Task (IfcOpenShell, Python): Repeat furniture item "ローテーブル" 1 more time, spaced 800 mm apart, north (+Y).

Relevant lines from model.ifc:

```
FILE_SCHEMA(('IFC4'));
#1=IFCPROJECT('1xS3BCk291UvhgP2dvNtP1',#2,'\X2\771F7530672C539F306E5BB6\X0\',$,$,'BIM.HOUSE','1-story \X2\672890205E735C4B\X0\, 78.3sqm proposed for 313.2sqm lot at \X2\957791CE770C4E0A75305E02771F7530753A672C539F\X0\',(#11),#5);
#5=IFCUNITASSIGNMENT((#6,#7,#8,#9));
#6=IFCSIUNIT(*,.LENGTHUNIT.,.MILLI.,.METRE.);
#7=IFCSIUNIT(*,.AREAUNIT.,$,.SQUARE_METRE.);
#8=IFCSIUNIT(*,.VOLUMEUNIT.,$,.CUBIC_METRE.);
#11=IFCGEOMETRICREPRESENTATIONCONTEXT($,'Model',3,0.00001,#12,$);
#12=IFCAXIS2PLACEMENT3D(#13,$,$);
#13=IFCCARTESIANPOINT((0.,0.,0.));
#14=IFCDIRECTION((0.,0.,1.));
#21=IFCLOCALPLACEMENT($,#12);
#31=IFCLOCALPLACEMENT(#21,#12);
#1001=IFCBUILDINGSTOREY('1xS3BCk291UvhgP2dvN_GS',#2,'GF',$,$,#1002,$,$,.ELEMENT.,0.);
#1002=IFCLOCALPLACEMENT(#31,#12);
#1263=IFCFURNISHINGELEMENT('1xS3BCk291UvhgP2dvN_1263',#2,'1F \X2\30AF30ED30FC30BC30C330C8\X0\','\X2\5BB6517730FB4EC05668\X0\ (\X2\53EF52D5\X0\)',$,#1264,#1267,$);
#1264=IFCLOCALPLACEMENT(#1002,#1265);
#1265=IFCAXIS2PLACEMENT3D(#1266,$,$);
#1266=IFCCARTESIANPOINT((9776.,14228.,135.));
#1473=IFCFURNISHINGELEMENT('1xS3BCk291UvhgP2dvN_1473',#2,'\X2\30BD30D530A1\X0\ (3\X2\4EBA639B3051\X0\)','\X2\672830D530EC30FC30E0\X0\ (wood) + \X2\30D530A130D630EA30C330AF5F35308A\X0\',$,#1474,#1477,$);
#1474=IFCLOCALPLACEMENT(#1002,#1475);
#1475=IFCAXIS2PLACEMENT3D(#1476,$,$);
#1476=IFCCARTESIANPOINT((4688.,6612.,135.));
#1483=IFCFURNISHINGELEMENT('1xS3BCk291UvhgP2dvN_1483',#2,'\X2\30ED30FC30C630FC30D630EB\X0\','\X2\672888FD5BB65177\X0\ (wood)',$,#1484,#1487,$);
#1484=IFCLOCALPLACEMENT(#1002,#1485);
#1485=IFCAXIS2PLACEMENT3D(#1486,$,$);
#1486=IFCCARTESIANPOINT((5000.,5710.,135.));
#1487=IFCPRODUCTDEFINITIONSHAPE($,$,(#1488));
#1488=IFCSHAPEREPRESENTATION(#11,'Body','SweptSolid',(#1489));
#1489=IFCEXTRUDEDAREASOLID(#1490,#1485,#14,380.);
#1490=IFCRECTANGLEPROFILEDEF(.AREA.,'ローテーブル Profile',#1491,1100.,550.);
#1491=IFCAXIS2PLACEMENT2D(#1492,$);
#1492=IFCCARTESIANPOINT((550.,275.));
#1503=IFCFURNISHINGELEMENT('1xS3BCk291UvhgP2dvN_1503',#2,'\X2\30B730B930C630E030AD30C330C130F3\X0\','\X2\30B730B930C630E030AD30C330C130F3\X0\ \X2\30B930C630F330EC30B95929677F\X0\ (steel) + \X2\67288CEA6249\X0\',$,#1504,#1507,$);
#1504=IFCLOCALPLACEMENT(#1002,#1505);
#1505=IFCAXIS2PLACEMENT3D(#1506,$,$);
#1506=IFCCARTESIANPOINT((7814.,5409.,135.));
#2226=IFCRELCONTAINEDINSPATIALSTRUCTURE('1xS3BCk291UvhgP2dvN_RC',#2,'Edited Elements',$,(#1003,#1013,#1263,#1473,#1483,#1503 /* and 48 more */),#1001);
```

```python
import numpy as np
import ifcopenshell
import ifcopenshell.api.geometry
import ifcopenshell.api.root
import ifcopenshell.util.element
import ifcopenshell.util.placement

model = ifcopenshell.open("model.ifc")


def reuse_history(source, copy):
    """copy_class also copies each property set's owner history, people and application; keep the originals."""
    for rel in copy.IsDefinedBy:
        if rel.is_a("IfcRelDefinesByProperties") and (history := rel.RelatingPropertyDefinition.OwnerHistory):
            rel.RelatingPropertyDefinition.OwnerHistory = source.OwnerHistory
            ifcopenshell.util.element.remove_deep2(model, history)


source = model.by_id(1483)
base = ifcopenshell.util.placement.get_local_placement(source.ObjectPlacement)
step = np.array([0.0, 1.0, 0.0]) * 800.0

for i in range(1, 2):
    copy = ifcopenshell.api.root.copy_class(model, product=source)
    copy.Representation = ifcopenshell.util.element.copy_deep(
        model, source.Representation, exclude=["IfcGeometricRepresentationContext", "IfcRepresentationMap"]
    )
    reuse_history(source, copy)
    matrix = base.copy()
    matrix[:3, 3] += i * step
    print("added at", matrix[:3, 3].round(3) + 0.0)
    ifcopenshell.api.geometry.edit_object_placement(model, product=copy, matrix=matrix, is_si=False)

model.write("model_edited.ifc")
```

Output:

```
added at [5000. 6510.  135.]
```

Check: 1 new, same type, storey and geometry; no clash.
